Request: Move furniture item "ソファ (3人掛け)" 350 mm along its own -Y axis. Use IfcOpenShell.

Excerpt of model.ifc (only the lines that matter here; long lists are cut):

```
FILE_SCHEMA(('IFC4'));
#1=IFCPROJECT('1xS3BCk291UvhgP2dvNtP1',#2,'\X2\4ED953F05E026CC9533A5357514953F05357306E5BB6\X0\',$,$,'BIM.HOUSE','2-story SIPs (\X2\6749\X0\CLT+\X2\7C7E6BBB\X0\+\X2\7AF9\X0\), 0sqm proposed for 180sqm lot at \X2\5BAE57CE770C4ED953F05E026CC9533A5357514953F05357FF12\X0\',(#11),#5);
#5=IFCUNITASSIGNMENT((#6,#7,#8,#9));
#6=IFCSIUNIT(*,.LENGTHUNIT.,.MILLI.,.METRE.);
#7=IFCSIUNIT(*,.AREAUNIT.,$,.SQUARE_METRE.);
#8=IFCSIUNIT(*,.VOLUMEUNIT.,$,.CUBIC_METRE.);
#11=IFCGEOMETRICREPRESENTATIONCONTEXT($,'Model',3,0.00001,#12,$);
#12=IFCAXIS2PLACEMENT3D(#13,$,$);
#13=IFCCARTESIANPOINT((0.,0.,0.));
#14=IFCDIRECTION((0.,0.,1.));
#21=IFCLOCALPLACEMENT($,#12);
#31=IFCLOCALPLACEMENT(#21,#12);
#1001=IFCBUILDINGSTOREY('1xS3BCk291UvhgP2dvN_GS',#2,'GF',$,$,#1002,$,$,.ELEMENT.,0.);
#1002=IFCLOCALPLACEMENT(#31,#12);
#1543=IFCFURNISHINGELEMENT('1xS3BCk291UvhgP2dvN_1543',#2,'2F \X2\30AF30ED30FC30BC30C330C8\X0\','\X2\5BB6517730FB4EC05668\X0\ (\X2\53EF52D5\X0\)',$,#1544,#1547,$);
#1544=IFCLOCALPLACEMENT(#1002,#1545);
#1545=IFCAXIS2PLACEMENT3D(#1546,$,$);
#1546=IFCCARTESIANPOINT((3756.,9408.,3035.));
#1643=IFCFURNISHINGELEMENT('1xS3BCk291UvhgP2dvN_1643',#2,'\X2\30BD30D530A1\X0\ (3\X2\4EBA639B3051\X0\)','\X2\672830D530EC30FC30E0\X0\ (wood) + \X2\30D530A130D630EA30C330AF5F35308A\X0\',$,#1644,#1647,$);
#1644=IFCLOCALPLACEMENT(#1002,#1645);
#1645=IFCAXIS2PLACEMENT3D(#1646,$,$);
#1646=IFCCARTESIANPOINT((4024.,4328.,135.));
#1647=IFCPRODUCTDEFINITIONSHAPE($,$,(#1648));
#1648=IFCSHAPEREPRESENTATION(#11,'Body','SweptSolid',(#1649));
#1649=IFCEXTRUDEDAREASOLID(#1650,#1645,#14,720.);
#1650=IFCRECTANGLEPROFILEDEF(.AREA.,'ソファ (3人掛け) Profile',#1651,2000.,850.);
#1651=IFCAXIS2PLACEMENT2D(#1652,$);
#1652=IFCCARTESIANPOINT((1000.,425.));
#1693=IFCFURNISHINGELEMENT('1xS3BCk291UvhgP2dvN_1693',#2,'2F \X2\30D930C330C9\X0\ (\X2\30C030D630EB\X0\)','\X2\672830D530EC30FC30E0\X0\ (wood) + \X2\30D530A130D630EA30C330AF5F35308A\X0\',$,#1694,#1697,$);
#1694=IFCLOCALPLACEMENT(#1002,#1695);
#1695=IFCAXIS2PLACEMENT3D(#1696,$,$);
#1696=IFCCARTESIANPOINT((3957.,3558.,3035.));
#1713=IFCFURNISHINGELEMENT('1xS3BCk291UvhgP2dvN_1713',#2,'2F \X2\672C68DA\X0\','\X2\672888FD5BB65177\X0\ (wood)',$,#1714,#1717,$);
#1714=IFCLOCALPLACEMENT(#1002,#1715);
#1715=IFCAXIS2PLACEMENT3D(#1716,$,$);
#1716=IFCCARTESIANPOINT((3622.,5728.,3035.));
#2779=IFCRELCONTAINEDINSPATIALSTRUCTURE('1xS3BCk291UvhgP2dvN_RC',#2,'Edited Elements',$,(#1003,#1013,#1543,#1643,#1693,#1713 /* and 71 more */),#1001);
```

```python
import ifcopenshell
import ifcopenshell.api.geometry
import ifcopenshell.util.placement

model = ifcopenshell.open("model.ifc")

item = model.by_guid("1xS3BCk291UvhgP2dvN_1643")
matrix = ifcopenshell.util.placement.get_local_placement(item.ObjectPlacement)
matrix[:3, 3] -= matrix[:3, 1] * 350.0
ifcopenshell.api.geometry.edit_object_placement(model, product=item, matrix=matrix, is_si=False)

print(ifcopenshell.util.placement.get_local_placement(item.ObjectPlacement).round(3) + 0.0)

model.write("model_edited.ifc")
```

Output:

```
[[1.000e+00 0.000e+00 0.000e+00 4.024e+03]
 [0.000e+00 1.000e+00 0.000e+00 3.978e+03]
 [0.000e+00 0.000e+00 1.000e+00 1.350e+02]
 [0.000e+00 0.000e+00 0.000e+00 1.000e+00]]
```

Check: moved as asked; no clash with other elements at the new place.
